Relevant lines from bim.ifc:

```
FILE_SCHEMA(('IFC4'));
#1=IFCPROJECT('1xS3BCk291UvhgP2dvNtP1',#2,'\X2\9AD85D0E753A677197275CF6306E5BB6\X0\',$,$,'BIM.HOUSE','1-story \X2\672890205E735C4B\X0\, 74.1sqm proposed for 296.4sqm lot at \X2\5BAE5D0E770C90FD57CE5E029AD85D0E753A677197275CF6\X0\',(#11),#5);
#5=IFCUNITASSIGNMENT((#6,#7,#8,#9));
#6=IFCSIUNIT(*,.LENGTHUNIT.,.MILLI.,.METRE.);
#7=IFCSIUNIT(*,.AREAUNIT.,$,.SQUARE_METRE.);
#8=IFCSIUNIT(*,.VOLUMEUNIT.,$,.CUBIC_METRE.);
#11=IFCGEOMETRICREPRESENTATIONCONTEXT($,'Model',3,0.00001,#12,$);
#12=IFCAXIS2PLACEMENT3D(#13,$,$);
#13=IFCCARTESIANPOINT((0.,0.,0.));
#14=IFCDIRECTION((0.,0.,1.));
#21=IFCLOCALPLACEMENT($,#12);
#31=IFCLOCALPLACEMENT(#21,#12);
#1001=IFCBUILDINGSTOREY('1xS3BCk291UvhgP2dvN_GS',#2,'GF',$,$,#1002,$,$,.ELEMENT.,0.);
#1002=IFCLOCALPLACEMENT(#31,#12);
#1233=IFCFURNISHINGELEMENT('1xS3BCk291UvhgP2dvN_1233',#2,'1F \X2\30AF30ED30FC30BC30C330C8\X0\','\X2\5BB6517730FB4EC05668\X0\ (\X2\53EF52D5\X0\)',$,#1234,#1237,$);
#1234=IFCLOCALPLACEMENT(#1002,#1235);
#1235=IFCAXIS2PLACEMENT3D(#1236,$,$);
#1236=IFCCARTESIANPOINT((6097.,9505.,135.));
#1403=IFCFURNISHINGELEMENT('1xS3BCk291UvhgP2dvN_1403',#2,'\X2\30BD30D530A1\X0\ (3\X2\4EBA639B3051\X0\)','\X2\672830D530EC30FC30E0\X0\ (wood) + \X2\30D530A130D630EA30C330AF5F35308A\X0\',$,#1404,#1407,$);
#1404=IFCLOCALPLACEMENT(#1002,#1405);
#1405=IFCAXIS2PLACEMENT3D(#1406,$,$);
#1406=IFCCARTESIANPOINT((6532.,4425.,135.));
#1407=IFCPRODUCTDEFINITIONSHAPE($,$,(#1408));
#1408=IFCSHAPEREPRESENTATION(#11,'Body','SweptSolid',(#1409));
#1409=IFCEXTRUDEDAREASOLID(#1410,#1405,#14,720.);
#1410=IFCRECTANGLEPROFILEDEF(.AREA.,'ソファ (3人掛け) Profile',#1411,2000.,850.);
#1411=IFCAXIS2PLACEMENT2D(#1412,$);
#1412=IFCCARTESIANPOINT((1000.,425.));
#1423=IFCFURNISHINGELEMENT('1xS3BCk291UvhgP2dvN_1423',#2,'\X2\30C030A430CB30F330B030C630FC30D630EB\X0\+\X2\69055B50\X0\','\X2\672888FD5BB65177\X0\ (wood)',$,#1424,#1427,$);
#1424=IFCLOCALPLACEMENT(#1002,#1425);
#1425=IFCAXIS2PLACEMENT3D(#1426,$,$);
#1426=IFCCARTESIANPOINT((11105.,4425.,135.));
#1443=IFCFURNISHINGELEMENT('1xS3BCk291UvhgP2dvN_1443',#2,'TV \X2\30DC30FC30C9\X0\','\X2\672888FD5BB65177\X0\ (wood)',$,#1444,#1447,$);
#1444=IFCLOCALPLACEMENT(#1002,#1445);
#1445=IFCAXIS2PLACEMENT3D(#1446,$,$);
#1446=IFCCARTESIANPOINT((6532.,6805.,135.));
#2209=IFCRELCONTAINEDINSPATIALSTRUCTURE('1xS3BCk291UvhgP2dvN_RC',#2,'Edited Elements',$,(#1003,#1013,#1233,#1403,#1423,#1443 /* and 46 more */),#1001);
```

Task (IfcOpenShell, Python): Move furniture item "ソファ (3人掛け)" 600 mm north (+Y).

```python
import ifcopenshell
import ifcopenshell.api.geometry
import ifcopenshell.util.placement
import ifcopenshell.util.unit

model = ifcopenshell.open("bim.ifc")
unit_scale = ifcopenshell.util.unit.calculate_unit_scale(model)

item = model.by_guid("1xS3BCk291UvhgP2dvN_1403")
matrix = ifcopenshell.util.placement.get_local_placement(item.ObjectPlacement)
matrix[1, 3] += 0.6 / unit_scale
ifcopenshell.api.geometry.edit_object_placement(model, product=item, matrix=matrix, is_si=False)

print(ifcopenshell.util.placement.get_local_placement(item.ObjectPlacement).round(3) + 0.0)

model.write("bim_edited.ifc")
```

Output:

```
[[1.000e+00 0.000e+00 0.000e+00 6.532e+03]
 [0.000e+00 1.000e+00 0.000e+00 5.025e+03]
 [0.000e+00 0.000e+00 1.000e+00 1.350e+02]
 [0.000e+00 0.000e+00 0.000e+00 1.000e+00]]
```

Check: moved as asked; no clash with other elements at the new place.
